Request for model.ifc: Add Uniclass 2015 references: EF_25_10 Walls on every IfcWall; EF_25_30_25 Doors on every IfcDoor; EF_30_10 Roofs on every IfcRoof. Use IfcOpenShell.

First a look at what the model holds.

```python
import ifcopenshell

model = ifcopenshell.open("model.ifc")
print(model.schema)
print("classifications:", [c.Name for c in model.by_type("IfcClassification")])
for ifc_class in ("IfcDoor", "IfcRoof", "IfcStair", "IfcWall", "IfcWindow"):
    print(ifc_class, len(model.by_type(ifc_class)))
```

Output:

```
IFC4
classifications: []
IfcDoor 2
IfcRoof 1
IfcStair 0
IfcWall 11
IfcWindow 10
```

```python
import ifcopenshell
import ifcopenshell.api.classification

model = ifcopenshell.open("model.ifc")

system = ifcopenshell.api.classification.add_classification(model, classification="Uniclass 2015")

codes = {
    "IfcWall": ("EF_25_10", "Walls"),
    "IfcDoor": ("EF_25_30_25", "Doors"),
    "IfcRoof": ("EF_30_10", "Roofs"),
}
for ifc_class, (code, name) in codes.items():
    products = model.by_type(ifc_class)
    ifcopenshell.api.classification.add_reference(
        model, products=products, classification=system, identification=code, name=name
    )
    print(code, len(products))

model.write("model-out.ifc")
```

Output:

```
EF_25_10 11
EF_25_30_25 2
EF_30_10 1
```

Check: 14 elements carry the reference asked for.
